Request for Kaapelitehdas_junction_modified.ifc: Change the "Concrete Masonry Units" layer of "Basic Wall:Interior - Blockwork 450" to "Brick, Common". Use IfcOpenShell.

First a look at what the model holds.

```python
import ifcopenshell
import ifcopenshell.util.element

model = ifcopenshell.open("Kaapelitehdas_junction_modified.ifc")
print(model.schema)
for layer_set in model.by_type("IfcMaterialLayerSet"):
    if layer_set.LayerSetName == "Basic Wall:Interior - Blockwork 450":
        for layer in layer_set.MaterialLayers:
            print(layer.id(), layer.Material and layer.Material.Name, layer.LayerThickness, sep=" | ")
        print(len(ifcopenshell.util.element.get_elements_by_material(model, layer_set)), "elements and types use it")
print(sorted(m.Name for m in model.by_type("IfcMaterial") if m.Name)[:60])
```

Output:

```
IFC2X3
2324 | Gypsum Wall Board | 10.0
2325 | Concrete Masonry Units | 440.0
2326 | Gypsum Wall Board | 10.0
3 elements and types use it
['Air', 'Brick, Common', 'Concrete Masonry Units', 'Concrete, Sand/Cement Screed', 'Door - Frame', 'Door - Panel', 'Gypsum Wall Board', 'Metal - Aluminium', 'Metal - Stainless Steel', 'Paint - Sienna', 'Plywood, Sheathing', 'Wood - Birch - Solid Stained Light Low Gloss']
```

```python
import ifcopenshell
import ifcopenshell.api.material

model = ifcopenshell.open("Kaapelitehdas_junction_modified.ifc")

layer_set = next(s for s in model.by_type("IfcMaterialLayerSet") if s.LayerSetName == "Basic Wall:Interior - Blockwork 450")
layer = next(l for l in layer_set.MaterialLayers if l.Material and l.Material.Name == "Concrete Masonry Units")
material = next(m for m in model.by_type("IfcMaterial") if m.Name == "Brick, Common")

# Point this one layer at the other material; renaming the old one would change it everywhere.
ifcopenshell.api.material.edit_layer(model, layer=layer, attributes={}, material=material)

print([l.Material.Name if l.Material else None for l in layer_set.MaterialLayers])

model.write("Kaapelitehdas_junction_modified_rev.ifc")
```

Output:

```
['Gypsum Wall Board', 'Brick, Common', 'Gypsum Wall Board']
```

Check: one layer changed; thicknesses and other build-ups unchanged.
